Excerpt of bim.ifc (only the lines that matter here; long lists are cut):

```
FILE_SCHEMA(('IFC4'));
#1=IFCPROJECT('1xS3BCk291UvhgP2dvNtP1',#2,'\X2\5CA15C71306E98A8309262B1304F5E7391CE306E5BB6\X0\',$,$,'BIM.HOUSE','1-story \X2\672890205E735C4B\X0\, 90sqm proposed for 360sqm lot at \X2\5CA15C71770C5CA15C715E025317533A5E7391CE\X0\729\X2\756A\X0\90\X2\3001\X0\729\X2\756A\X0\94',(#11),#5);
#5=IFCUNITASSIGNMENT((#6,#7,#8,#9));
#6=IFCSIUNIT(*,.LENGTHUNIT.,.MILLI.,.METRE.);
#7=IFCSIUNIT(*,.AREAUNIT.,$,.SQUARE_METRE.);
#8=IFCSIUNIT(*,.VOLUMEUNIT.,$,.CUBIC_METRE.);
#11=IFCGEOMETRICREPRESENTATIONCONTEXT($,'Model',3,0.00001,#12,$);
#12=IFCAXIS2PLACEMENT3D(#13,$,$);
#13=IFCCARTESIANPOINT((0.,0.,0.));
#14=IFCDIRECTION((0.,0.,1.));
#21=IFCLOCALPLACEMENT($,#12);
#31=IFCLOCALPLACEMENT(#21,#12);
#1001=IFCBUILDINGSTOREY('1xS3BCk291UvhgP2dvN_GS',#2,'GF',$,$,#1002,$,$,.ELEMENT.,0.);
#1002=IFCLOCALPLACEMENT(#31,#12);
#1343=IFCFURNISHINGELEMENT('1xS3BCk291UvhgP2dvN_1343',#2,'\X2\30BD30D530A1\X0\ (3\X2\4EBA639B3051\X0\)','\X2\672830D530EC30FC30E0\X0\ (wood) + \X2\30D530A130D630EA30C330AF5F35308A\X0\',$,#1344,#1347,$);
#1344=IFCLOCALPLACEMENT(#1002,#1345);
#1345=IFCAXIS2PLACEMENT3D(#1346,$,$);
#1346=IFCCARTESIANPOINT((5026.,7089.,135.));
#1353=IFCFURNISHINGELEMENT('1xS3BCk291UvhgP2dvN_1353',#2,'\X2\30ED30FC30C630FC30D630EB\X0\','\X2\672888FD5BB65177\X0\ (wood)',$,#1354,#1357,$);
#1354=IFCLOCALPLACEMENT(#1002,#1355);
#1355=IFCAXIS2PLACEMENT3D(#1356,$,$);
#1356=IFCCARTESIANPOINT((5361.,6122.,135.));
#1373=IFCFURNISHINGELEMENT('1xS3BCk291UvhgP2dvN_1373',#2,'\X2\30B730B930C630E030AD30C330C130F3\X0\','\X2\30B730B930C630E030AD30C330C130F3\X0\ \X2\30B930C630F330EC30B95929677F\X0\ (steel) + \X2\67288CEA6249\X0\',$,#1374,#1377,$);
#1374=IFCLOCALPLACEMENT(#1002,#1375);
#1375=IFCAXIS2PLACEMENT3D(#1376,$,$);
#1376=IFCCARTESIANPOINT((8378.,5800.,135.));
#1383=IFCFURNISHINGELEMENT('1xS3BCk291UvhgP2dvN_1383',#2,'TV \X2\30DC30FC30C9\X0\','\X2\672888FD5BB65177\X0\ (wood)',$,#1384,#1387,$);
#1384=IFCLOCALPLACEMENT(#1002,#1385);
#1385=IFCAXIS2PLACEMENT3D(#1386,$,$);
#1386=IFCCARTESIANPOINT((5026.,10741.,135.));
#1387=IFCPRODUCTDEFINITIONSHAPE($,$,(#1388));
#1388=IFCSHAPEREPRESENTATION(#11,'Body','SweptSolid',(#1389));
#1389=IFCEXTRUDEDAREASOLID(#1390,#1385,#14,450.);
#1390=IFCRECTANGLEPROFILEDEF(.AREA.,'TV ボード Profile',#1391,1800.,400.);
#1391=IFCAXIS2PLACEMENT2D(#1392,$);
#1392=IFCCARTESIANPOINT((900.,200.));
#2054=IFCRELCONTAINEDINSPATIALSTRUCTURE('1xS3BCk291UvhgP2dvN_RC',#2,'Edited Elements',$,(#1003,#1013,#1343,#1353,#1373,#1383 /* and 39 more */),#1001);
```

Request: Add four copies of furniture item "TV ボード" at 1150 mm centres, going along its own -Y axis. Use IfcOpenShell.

```python
import ifcopenshell
import ifcopenshell.api.geometry
import ifcopenshell.api.root
import ifcopenshell.util.element
import ifcopenshell.util.placement

model = ifcopenshell.open("bim.ifc")


def reuse_history(source, copy):
    """copy_class also copies each property set's owner history, people and application; keep the originals."""
    for rel in copy.IsDefinedBy:
        if rel.is_a("IfcRelDefinesByProperties") and (history := rel.RelatingPropertyDefinition.OwnerHistory):
            rel.RelatingPropertyDefinition.OwnerHistory = source.OwnerHistory
            ifcopenshell.util.element.remove_deep2(model, history)


source = model.by_guid("1xS3BCk291UvhgP2dvN_1383")
base = ifcopenshell.util.placement.get_local_placement(source.ObjectPlacement)
step = -base[:3, 1] * 1150.0

for i in range(1, 5):
    copy = ifcopenshell.api.root.copy_class(model, product=source)
    copy.Representation = ifcopenshell.util.element.copy_deep(
        model, source.Representation, exclude=["IfcGeometricRepresentationContext", "IfcRepresentationMap"]
    )
    reuse_history(source, copy)
    matrix = base.copy()
    matrix[:3, 3] += i * step
    print("added at", matrix[:3, 3].round(3) + 0.0)
    ifcopenshell.api.geometry.edit_object_placement(model, product=copy, matrix=matrix, is_si=False)

model.write("bim_v2.ifc")
```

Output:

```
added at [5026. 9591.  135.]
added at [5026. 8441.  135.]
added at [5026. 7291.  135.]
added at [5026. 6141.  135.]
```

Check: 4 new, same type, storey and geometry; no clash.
